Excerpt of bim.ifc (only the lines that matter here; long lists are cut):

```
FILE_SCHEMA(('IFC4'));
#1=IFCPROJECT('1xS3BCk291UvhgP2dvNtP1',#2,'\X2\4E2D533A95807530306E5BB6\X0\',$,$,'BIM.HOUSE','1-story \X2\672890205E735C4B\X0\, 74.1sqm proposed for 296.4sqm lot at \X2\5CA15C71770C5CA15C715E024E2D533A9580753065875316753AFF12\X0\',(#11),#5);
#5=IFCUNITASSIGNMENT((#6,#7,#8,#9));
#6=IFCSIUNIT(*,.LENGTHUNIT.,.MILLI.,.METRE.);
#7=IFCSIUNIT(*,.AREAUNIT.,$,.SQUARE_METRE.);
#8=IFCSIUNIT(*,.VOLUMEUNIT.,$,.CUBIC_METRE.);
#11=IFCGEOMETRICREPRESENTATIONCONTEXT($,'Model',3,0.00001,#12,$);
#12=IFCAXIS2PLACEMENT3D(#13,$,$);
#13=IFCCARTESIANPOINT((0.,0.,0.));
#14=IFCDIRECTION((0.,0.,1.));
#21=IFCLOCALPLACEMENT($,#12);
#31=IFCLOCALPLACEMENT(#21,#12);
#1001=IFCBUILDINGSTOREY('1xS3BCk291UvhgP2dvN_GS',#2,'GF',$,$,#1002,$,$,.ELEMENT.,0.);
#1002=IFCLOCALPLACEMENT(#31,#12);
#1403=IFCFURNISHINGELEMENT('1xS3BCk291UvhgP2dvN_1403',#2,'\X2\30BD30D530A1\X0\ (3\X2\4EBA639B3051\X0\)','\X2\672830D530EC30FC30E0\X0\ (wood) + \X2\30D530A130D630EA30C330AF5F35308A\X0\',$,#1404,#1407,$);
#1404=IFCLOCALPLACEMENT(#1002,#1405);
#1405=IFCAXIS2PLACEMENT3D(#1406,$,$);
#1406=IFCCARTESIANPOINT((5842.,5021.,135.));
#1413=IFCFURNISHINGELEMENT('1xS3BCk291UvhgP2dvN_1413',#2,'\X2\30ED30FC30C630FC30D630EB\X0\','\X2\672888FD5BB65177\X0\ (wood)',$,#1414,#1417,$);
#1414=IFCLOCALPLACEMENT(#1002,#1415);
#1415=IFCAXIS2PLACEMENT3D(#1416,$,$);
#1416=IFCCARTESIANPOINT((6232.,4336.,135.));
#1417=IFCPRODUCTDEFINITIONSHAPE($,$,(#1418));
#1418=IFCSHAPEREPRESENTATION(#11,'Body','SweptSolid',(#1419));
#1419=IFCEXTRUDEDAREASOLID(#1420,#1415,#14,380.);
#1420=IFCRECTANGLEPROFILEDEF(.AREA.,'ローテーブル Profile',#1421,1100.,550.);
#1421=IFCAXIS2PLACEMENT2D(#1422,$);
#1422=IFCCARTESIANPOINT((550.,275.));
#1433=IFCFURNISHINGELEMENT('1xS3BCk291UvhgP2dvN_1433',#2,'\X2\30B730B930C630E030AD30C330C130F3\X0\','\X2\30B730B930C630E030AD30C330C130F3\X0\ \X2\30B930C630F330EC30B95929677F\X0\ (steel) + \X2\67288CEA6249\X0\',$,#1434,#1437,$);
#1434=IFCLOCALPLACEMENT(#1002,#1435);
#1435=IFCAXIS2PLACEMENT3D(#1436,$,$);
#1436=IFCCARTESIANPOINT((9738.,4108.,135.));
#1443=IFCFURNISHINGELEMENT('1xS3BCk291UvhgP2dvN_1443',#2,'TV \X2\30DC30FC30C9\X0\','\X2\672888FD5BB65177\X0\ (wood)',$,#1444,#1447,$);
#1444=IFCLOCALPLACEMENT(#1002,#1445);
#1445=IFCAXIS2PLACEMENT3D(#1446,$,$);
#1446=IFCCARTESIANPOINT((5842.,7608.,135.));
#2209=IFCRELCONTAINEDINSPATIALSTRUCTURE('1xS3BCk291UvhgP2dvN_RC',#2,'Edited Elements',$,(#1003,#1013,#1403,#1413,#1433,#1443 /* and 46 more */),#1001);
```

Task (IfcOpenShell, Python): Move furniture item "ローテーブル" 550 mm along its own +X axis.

```python
import ifcopenshell
import ifcopenshell.api.geometry
import ifcopenshell.util.placement
import ifcopenshell.util.unit

model = ifcopenshell.open("bim.ifc")
unit_scale = ifcopenshell.util.unit.calculate_unit_scale(model)

item = model.by_id(1413)
matrix = ifcopenshell.util.placement.get_local_placement(item.ObjectPlacement)
matrix[:3, 3] += matrix[:3, 0] * 0.55 / unit_scale
ifcopenshell.api.geometry.edit_object_placement(model, product=item, matrix=matrix, is_si=False)

print(ifcopenshell.util.placement.get_local_placement(item.ObjectPlacement).round(3) + 0.0)

model.write("bim_rev.ifc")
```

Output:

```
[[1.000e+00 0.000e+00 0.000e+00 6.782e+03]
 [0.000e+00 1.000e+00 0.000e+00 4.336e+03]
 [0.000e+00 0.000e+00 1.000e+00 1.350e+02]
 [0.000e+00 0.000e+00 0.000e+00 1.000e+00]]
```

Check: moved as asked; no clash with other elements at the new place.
